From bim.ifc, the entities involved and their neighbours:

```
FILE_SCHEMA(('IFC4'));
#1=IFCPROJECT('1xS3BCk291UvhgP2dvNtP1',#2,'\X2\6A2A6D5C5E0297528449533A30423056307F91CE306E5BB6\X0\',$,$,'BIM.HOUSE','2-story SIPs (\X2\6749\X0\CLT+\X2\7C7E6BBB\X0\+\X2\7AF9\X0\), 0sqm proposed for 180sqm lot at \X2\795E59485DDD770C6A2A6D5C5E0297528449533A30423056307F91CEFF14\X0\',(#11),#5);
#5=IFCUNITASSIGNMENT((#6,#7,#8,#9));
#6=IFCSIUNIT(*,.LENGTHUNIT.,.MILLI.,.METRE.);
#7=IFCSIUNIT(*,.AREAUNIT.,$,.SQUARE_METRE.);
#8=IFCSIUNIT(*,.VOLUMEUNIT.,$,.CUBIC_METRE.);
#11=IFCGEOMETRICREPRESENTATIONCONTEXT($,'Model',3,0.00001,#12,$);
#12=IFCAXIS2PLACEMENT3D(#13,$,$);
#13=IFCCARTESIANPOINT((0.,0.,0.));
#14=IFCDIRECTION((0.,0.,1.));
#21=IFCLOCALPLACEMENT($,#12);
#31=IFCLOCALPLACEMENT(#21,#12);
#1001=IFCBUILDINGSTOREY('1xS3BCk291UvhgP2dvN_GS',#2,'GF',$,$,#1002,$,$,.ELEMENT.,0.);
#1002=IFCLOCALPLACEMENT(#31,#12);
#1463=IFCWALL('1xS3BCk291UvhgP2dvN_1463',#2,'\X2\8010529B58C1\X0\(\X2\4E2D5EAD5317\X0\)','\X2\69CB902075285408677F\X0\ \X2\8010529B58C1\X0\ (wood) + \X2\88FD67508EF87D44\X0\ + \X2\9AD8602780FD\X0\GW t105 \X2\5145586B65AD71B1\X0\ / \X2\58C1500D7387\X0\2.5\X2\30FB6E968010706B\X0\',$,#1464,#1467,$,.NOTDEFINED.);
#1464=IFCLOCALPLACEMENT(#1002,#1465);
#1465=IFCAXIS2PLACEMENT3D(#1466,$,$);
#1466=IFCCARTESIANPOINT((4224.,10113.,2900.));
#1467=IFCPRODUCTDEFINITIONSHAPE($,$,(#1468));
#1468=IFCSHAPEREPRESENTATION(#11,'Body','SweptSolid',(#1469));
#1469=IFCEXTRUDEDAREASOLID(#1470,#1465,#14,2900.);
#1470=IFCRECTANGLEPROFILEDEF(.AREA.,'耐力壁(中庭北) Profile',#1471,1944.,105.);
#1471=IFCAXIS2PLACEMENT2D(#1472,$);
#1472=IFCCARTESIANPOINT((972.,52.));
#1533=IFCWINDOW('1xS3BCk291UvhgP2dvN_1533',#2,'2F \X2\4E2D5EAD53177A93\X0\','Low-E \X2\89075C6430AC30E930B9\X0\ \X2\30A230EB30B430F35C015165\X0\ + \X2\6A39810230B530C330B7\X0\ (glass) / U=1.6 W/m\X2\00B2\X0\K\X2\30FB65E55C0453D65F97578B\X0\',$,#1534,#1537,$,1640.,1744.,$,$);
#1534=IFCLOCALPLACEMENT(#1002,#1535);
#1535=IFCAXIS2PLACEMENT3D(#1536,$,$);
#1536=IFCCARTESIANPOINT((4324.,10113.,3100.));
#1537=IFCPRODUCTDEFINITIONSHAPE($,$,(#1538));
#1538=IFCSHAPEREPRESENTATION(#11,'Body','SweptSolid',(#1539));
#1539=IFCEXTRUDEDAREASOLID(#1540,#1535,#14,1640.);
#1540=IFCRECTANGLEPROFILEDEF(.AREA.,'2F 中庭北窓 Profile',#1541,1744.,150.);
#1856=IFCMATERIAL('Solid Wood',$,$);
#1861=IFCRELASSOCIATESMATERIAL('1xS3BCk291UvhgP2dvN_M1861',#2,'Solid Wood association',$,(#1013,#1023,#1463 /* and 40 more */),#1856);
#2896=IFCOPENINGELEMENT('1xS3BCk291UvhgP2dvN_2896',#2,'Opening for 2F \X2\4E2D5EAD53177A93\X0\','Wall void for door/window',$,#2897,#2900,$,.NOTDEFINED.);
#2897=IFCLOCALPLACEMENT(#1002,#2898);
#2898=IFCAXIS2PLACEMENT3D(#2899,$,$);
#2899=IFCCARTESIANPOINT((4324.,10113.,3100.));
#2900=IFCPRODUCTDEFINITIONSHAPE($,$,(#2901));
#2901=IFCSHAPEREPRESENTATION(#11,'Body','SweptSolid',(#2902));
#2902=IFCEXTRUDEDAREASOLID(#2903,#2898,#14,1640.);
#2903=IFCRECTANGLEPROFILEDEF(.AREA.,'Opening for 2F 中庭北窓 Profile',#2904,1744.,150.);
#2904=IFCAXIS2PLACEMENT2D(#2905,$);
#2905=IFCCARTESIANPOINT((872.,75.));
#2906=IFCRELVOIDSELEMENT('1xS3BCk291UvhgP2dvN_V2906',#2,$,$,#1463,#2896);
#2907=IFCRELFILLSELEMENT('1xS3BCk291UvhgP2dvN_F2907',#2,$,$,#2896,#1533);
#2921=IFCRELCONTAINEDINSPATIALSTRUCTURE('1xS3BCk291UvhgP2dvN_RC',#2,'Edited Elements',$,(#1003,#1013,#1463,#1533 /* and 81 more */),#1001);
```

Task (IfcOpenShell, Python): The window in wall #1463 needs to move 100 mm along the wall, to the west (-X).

```python
import ifcopenshell
import ifcopenshell.api.geometry
import ifcopenshell.util.placement

model = ifcopenshell.open("bim.ifc")

window = model.by_guid("1xS3BCk291UvhgP2dvN_1533")
opening = window.FillsVoids[0].RelatingOpeningElement
wall = opening.VoidsElements[0].RelatingBuildingElement

wall_matrix = ifcopenshell.util.placement.get_local_placement(wall.ObjectPlacement)
shift = wall_matrix[:3, 0] * -100.0
before = ifcopenshell.util.placement.get_local_placement(window.ObjectPlacement)[:3, 3].copy()

# The window is not placed relative to its opening, so move both.
for product in (opening, window):
    matrix = ifcopenshell.util.placement.get_local_placement(product.ObjectPlacement)
    matrix[:3, 3] += shift
    ifcopenshell.api.geometry.edit_object_placement(model, product=product, matrix=matrix, is_si=False)

after = ifcopenshell.util.placement.get_local_placement(window.ObjectPlacement)[:3, 3]
print("window moved by", (after - before).round(3) + 0.0)

model.write("bim-out.ifc")
```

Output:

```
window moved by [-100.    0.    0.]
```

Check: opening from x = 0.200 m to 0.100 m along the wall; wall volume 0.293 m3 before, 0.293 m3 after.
